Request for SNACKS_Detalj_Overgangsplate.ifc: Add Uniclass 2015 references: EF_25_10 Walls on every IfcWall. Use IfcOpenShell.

First a look at what the model holds.

```python
import ifcopenshell

model = ifcopenshell.open("SNACKS_Detalj_Overgangsplate.ifc")
print(model.schema)
print("classifications:", [c.Name for c in model.by_type("IfcClassification")])
for ifc_class in ("IfcDoor", "IfcRoof", "IfcStair", "IfcWall", "IfcWindow"):
    print(ifc_class, len(model.by_type(ifc_class)))
```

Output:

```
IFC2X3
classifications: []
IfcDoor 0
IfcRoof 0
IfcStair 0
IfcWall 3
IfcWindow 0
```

```python
import ifcopenshell
import ifcopenshell.api.classification

model = ifcopenshell.open("SNACKS_Detalj_Overgangsplate.ifc")

# IFC2X3 requires Source and Edition and has no link from the project to the system.
system = model.create_entity("IfcClassification", Source="NBS", Edition="2015", Name="Uniclass 2015")

codes = {
    "IfcWall": ("EF_25_10", "Walls"),
}
for ifc_class, (code, name) in codes.items():
    products = model.by_type(ifc_class)
    ifcopenshell.api.classification.add_reference(
        model, products=products, classification=system, identification=code, name=name
    )
    print(code, len(products))

model.write("SNACKS_Detalj_Overgangsplate_updated.ifc")
```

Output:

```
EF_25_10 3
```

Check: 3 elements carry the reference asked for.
